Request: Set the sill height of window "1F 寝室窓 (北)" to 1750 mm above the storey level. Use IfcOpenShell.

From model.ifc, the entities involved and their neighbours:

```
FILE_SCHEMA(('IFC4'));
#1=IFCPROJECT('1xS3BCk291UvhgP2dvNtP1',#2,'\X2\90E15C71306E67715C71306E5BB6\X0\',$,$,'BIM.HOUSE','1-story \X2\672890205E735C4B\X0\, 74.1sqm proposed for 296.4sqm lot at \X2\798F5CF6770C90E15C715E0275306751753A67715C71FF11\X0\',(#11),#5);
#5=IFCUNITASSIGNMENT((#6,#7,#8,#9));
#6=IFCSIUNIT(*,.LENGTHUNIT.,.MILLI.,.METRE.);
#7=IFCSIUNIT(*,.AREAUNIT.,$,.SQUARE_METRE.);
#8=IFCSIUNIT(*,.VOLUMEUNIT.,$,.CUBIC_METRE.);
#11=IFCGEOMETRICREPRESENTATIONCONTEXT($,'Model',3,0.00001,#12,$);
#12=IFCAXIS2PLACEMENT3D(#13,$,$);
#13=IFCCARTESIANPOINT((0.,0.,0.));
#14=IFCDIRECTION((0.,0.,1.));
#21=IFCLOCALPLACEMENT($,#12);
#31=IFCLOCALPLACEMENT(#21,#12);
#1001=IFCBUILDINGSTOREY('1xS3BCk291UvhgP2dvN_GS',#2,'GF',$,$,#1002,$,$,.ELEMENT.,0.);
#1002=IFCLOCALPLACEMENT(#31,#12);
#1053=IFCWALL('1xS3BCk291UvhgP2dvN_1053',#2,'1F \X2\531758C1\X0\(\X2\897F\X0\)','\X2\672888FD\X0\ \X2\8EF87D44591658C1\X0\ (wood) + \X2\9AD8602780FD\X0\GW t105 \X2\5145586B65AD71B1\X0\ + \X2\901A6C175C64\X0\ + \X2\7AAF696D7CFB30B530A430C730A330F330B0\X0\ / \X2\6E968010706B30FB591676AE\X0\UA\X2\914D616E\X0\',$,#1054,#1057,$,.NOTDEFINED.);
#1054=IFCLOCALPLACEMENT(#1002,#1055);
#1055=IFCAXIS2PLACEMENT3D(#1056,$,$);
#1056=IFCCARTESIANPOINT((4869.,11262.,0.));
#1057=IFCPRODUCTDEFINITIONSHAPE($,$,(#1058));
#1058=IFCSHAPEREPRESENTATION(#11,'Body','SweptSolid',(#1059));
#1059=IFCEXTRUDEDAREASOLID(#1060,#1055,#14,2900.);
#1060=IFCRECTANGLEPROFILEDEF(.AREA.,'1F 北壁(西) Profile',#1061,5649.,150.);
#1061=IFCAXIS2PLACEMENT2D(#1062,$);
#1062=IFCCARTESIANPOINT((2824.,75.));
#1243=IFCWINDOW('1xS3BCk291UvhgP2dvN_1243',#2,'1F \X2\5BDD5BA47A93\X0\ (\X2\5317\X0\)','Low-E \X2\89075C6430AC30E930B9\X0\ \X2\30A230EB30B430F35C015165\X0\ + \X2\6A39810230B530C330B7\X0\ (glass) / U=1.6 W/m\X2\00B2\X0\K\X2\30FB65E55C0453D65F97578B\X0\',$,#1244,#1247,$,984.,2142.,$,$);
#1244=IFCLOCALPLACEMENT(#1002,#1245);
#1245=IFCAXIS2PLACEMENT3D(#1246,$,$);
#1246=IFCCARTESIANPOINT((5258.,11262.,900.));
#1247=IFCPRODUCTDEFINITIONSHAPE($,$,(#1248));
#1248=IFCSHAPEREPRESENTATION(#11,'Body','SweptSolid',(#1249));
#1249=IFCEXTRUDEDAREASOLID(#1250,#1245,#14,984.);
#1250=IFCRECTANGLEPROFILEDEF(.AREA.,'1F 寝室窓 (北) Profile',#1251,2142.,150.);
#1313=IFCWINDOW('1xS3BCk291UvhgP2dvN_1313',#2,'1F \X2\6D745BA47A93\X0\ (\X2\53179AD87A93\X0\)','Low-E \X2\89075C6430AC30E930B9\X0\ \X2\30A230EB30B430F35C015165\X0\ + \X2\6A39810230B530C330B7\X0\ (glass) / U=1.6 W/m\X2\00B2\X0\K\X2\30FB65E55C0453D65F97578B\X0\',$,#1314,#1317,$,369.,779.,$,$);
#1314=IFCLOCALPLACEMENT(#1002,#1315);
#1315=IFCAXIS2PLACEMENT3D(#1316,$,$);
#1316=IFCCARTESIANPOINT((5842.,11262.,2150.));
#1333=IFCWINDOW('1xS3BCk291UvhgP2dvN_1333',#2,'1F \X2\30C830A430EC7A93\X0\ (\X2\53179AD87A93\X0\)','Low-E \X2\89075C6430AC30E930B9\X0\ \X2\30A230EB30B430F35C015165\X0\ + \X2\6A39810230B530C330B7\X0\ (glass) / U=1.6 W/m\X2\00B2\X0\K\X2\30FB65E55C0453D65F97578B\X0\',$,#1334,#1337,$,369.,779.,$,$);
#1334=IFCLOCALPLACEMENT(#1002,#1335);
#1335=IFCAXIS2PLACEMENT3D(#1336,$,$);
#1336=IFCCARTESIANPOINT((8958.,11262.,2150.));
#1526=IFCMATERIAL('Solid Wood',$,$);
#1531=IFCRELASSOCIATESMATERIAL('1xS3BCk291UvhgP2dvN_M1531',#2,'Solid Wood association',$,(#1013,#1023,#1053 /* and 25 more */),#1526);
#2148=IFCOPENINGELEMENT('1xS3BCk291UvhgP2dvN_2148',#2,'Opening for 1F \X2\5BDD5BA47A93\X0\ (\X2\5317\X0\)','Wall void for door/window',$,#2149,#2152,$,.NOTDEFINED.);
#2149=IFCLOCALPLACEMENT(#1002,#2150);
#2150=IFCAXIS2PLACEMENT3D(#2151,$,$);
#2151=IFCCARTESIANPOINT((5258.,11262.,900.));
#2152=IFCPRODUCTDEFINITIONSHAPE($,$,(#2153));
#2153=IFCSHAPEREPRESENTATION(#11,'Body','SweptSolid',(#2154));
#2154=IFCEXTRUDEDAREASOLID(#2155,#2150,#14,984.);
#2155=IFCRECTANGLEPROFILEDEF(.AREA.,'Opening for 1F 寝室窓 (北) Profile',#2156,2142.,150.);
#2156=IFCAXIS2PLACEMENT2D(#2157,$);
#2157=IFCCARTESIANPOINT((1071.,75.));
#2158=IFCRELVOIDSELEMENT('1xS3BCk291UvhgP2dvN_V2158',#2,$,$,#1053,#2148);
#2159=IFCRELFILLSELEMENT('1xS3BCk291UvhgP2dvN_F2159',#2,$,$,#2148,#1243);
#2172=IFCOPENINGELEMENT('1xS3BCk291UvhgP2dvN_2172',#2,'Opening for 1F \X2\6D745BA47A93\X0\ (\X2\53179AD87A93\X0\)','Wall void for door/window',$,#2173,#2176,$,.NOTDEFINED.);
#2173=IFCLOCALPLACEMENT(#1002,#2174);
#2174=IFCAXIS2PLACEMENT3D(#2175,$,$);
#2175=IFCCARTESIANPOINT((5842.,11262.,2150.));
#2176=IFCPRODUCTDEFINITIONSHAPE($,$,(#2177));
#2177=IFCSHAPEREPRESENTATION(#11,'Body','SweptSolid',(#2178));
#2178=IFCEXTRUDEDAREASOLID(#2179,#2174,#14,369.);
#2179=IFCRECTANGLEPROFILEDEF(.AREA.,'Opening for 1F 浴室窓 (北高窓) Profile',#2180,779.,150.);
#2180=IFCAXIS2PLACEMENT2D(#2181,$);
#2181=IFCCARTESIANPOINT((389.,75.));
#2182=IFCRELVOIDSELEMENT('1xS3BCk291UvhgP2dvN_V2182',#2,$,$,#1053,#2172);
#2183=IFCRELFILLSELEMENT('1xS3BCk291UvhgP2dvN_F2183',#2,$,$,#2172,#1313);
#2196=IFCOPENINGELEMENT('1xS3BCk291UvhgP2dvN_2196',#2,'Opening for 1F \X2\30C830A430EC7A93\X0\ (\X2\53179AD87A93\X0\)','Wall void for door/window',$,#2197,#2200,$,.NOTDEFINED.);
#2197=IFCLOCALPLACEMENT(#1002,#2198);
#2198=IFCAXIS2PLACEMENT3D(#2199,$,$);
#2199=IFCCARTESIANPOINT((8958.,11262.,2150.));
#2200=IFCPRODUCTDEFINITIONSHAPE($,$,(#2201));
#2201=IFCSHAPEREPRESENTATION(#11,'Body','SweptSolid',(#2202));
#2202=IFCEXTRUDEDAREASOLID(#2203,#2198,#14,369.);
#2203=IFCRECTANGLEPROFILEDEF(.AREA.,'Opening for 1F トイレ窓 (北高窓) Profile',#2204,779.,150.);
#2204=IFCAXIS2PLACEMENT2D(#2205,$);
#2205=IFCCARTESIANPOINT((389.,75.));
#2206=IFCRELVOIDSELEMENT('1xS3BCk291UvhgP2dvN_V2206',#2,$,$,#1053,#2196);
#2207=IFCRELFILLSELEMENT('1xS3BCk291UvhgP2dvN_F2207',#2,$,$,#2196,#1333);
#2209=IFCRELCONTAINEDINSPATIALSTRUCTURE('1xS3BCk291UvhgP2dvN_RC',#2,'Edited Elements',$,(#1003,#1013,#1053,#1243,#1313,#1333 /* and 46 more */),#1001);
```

```python
import numpy as np
import ifcopenshell
import ifcopenshell.api.geometry
import ifcopenshell.geom
import ifcopenshell.util.element
import ifcopenshell.util.placement
import ifcopenshell.util.shape
import ifcopenshell.util.unit

model = ifcopenshell.open("model.ifc")
unit_scale = ifcopenshell.util.unit.calculate_unit_scale(model)

window = model.by_id(1243)
opening = window.FillsVoids[0].RelatingOpeningElement
storey = ifcopenshell.util.element.get_container(window, ifc_class="IfcBuildingStorey")
level = ifcopenshell.util.placement.get_local_placement(storey.ObjectPlacement)[2, 3]

# The opening's origin need not be at the sill, so measure its lowest point.
shape = ifcopenshell.geom.create_shape(ifcopenshell.geom.settings(), opening)
bottom = ifcopenshell.util.shape.get_shape_bottom_elevation(shape, shape.geometry) / unit_scale
dz = level + 1750.0 - bottom

shift = np.array([0.0, 0.0, dz])
# The window is not placed relative to its opening, so move both.
for product in (opening, window):
    matrix = ifcopenshell.util.placement.get_local_placement(product.ObjectPlacement)
    matrix[:3, 3] += shift
    ifcopenshell.api.geometry.edit_object_placement(model, product=product, matrix=matrix, is_si=False)

print(f"moved by {dz * unit_scale:+.3f} m")

model.write("model_v2.ifc")
```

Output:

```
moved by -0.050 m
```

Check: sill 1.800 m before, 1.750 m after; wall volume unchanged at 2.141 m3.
